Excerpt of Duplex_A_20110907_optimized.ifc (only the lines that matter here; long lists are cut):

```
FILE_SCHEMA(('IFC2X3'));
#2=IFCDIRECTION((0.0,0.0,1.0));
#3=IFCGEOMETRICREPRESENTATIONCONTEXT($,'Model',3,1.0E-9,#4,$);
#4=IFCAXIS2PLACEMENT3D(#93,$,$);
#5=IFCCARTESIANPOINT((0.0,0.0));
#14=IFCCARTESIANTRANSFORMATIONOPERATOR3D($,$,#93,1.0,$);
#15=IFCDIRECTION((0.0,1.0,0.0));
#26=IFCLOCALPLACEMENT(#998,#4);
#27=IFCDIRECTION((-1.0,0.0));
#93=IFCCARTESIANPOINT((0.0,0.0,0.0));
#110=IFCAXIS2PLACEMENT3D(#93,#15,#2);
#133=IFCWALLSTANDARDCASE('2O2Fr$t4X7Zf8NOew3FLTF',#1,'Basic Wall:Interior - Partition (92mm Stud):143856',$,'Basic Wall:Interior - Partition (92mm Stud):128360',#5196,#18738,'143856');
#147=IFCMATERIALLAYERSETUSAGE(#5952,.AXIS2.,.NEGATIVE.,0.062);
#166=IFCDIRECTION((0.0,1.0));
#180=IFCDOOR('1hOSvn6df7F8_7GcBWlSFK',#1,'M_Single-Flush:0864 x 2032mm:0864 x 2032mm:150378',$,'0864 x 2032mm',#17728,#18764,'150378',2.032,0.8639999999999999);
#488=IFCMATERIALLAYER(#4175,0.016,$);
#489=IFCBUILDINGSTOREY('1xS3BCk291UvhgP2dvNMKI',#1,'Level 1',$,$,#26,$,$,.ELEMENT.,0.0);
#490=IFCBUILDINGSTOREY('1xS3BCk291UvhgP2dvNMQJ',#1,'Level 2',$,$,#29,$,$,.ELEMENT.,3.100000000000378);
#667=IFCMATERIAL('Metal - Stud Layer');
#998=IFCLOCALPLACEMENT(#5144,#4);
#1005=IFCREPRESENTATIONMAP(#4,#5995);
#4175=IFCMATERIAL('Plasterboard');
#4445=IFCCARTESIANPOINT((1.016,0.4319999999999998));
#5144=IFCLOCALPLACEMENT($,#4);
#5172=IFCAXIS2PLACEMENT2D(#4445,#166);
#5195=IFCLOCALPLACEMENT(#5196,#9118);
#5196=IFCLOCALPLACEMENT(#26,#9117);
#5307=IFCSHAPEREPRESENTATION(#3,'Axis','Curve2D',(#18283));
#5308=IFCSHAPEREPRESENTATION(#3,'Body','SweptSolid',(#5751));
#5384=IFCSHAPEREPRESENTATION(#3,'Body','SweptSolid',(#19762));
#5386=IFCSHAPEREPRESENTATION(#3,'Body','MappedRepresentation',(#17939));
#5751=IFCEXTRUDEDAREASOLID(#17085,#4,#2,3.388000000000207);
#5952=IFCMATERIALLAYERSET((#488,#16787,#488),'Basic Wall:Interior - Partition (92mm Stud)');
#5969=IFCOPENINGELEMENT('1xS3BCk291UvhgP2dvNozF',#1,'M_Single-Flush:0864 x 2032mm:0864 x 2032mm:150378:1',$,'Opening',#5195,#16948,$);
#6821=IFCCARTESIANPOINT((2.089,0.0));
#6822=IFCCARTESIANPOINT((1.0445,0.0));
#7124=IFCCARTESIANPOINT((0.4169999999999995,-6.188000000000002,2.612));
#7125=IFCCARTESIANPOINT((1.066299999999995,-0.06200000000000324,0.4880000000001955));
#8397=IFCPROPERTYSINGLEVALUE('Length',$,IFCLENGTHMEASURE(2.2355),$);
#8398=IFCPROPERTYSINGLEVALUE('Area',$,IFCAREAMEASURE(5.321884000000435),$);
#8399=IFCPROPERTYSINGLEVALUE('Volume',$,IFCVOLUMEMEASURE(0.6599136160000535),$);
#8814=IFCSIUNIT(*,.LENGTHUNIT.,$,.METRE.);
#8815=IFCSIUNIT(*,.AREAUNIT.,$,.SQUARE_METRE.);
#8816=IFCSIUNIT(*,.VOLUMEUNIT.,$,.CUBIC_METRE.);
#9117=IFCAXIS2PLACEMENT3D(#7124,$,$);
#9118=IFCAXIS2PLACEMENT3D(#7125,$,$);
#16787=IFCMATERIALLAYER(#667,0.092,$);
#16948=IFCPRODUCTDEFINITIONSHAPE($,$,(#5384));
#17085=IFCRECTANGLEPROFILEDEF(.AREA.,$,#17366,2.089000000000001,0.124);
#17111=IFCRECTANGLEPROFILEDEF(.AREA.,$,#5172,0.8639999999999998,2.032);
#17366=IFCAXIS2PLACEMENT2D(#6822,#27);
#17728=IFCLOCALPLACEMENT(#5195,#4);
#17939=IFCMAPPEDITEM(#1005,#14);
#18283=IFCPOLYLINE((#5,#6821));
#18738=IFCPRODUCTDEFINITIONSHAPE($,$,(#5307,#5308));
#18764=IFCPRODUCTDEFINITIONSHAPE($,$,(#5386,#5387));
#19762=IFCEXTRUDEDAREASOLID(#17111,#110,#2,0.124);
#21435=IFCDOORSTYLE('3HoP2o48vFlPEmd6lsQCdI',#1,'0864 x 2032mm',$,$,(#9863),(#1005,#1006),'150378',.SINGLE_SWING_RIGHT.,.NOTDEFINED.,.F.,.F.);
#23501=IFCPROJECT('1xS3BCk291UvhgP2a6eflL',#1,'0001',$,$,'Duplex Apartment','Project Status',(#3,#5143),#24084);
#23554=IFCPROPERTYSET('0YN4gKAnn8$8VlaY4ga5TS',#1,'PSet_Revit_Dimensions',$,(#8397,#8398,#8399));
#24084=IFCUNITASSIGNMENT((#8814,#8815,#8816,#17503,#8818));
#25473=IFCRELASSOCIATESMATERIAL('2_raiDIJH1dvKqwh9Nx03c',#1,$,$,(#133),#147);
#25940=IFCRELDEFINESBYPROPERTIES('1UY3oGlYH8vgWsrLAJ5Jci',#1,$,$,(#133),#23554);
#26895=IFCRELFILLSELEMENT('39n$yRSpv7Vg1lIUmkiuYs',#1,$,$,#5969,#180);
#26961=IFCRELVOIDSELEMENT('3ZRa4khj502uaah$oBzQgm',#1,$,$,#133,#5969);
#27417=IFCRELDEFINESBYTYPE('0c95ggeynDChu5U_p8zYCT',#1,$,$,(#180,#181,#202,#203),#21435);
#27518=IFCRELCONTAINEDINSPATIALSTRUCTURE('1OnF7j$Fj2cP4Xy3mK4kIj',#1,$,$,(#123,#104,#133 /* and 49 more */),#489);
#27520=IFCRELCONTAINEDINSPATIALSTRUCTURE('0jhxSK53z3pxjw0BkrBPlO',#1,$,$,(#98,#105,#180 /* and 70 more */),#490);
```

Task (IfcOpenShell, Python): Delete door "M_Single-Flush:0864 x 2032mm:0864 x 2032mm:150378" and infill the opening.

```python
import ifcopenshell
import ifcopenshell.api.feature
import ifcopenshell.api.pset
import ifcopenshell.api.root
import ifcopenshell.geom
import ifcopenshell.util.element
import ifcopenshell.util.shape
import ifcopenshell.util.unit

model = ifcopenshell.open("Duplex_A_20110907_optimized.ifc")
area_scale = ifcopenshell.util.unit.calculate_unit_scale(model, "AREAUNIT")
volume_scale = ifcopenshell.util.unit.calculate_unit_scale(model, "VOLUMEUNIT")
settings = ifcopenshell.geom.settings()


def volume(element):
    """Net volume in cubic metres, openings subtracted."""
    shape = ifcopenshell.geom.create_shape(settings, element)
    return ifcopenshell.util.shape.get_volume(shape.geometry)


door = model.by_id(180)
opening = door.FillsVoids[0].RelatingOpeningElement
wall = opening.VoidsElements[0].RelatingBuildingElement
before = volume(wall)

ifcopenshell.api.root.remove_product(model, product=door)
ifcopenshell.api.feature.remove_feature(model, feature=opening)

after = volume(wall)
thickness = 0.124  # wall thickness in metres

# Update the wall's stored quantities.
pset = model.by_id(ifcopenshell.util.element.get_pset(wall, "PSet_Revit_Dimensions", should_inherit=False)["id"])
ifcopenshell.api.pset.edit_pset(model, pset=pset, properties={
    "Area": model.create_entity("IfcAreaMeasure", after / thickness / area_scale),
    "Volume": model.create_entity("IfcVolumeMeasure", after / volume_scale),
})

print(f"wall volume {before:.3f} -> {after:.3f} m3")

model.write("Duplex_A_20110907_optimized_rev.ifc")
```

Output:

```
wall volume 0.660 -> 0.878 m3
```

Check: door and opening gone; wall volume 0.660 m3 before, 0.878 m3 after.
